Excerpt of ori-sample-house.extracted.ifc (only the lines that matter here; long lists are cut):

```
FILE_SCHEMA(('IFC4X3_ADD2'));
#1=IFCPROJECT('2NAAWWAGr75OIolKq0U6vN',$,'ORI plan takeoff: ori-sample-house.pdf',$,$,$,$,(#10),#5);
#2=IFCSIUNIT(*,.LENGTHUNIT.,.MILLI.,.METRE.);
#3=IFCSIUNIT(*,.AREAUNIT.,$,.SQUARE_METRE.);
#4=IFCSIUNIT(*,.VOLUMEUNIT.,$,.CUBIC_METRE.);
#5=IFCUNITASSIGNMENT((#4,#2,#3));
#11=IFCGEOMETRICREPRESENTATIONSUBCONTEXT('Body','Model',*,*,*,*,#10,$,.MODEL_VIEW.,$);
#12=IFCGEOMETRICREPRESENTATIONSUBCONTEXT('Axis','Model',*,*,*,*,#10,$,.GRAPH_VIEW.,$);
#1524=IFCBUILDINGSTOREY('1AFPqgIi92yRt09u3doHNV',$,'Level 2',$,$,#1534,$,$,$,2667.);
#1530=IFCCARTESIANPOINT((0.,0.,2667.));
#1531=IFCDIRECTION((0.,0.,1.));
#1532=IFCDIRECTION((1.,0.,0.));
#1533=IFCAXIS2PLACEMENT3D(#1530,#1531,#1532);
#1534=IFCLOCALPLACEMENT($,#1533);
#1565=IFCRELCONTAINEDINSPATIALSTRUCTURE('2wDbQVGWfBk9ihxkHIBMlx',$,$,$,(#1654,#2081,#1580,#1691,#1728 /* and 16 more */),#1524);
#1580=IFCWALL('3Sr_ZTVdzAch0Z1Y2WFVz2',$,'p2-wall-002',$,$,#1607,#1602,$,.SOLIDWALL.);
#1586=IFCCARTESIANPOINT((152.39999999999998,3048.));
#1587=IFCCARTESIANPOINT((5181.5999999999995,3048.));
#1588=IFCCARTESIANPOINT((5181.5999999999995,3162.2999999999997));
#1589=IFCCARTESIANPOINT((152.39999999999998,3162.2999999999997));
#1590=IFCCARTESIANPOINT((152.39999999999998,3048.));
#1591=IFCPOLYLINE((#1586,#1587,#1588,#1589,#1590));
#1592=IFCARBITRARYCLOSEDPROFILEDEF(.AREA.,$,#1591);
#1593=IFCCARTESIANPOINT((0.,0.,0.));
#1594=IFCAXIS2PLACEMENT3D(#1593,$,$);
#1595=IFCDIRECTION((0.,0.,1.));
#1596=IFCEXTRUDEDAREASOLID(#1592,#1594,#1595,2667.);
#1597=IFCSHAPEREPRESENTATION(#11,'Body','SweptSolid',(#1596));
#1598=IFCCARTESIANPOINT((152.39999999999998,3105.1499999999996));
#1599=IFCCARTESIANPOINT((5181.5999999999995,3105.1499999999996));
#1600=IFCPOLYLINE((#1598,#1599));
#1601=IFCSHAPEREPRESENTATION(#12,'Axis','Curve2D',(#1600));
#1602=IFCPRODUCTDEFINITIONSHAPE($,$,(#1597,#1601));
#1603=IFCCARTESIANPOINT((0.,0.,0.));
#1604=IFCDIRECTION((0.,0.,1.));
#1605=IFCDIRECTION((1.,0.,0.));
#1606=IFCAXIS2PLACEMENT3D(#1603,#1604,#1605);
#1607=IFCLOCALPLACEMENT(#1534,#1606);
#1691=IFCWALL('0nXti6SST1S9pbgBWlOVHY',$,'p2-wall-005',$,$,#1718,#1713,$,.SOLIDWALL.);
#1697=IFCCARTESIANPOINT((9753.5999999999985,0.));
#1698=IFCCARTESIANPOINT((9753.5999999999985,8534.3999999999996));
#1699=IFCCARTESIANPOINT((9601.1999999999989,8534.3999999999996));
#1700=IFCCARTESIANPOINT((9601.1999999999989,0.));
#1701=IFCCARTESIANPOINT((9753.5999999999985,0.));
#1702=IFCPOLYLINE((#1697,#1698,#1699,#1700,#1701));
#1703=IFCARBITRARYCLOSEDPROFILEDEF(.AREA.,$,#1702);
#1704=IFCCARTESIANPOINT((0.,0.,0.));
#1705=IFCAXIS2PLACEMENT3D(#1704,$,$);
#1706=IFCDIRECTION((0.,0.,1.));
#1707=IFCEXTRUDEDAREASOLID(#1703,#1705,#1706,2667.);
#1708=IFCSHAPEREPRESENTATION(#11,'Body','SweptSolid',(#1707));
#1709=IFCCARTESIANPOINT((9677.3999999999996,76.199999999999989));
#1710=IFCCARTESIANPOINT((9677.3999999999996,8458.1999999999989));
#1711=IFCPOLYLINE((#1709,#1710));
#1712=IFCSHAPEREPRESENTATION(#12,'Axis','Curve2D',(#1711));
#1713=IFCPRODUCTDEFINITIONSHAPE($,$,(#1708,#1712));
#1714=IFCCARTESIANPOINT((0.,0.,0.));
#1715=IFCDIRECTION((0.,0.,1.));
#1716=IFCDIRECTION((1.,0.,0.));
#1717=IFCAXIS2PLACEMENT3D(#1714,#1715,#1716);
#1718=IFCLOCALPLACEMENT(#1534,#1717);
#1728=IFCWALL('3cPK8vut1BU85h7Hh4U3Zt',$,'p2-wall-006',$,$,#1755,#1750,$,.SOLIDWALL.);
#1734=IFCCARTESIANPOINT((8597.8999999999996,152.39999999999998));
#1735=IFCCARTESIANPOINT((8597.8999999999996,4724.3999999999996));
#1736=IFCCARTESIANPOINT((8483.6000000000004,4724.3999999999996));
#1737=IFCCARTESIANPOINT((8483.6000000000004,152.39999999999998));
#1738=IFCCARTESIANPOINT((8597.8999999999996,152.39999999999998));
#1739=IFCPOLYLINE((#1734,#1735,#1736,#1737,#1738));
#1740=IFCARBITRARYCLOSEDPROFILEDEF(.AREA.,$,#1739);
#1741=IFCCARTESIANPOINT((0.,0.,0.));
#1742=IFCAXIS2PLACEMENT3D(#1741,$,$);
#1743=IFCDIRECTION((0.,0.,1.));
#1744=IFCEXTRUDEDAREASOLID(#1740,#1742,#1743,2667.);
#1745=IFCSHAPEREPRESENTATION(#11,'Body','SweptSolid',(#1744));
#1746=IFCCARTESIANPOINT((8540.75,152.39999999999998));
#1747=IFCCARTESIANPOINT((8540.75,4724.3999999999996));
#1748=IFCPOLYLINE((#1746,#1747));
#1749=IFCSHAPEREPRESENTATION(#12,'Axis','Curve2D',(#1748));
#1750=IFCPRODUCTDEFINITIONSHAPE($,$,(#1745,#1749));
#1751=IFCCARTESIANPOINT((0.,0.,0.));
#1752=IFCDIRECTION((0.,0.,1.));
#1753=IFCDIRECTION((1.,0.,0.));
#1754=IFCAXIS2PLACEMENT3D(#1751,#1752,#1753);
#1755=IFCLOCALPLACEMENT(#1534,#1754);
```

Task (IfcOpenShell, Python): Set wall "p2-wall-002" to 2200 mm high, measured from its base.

```python
import ifcopenshell
import ifcopenshell.geom
import ifcopenshell.util.representation
import ifcopenshell.util.shape
import ifcopenshell.util.unit

model = ifcopenshell.open("ori-sample-house.extracted.ifc")
unit_scale = ifcopenshell.util.unit.calculate_unit_scale(model)
settings = ifcopenshell.geom.settings()


def volume(element):
    """Net volume in cubic metres, openings subtracted."""
    shape = ifcopenshell.geom.create_shape(settings, element)
    return ifcopenshell.util.shape.get_volume(shape.geometry)


wall = model.by_guid("3Sr_ZTVdzAch0Z1Y2WFVz2")
before = volume(wall)

body = ifcopenshell.util.representation.get_representation(wall, "Model", "Body")
solid = body.Items[0]
old_height = solid.Depth
solid.Depth = 2.2 / unit_scale
after = volume(wall)

print(f"height {old_height:g} -> {solid.Depth:g}, volume {before:.3f} -> {after:.3f} m3")

model.write("ori-sample-house.extracted_updated.ifc")
```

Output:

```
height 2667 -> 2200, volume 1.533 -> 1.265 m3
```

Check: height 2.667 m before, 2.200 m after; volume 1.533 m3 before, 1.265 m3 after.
